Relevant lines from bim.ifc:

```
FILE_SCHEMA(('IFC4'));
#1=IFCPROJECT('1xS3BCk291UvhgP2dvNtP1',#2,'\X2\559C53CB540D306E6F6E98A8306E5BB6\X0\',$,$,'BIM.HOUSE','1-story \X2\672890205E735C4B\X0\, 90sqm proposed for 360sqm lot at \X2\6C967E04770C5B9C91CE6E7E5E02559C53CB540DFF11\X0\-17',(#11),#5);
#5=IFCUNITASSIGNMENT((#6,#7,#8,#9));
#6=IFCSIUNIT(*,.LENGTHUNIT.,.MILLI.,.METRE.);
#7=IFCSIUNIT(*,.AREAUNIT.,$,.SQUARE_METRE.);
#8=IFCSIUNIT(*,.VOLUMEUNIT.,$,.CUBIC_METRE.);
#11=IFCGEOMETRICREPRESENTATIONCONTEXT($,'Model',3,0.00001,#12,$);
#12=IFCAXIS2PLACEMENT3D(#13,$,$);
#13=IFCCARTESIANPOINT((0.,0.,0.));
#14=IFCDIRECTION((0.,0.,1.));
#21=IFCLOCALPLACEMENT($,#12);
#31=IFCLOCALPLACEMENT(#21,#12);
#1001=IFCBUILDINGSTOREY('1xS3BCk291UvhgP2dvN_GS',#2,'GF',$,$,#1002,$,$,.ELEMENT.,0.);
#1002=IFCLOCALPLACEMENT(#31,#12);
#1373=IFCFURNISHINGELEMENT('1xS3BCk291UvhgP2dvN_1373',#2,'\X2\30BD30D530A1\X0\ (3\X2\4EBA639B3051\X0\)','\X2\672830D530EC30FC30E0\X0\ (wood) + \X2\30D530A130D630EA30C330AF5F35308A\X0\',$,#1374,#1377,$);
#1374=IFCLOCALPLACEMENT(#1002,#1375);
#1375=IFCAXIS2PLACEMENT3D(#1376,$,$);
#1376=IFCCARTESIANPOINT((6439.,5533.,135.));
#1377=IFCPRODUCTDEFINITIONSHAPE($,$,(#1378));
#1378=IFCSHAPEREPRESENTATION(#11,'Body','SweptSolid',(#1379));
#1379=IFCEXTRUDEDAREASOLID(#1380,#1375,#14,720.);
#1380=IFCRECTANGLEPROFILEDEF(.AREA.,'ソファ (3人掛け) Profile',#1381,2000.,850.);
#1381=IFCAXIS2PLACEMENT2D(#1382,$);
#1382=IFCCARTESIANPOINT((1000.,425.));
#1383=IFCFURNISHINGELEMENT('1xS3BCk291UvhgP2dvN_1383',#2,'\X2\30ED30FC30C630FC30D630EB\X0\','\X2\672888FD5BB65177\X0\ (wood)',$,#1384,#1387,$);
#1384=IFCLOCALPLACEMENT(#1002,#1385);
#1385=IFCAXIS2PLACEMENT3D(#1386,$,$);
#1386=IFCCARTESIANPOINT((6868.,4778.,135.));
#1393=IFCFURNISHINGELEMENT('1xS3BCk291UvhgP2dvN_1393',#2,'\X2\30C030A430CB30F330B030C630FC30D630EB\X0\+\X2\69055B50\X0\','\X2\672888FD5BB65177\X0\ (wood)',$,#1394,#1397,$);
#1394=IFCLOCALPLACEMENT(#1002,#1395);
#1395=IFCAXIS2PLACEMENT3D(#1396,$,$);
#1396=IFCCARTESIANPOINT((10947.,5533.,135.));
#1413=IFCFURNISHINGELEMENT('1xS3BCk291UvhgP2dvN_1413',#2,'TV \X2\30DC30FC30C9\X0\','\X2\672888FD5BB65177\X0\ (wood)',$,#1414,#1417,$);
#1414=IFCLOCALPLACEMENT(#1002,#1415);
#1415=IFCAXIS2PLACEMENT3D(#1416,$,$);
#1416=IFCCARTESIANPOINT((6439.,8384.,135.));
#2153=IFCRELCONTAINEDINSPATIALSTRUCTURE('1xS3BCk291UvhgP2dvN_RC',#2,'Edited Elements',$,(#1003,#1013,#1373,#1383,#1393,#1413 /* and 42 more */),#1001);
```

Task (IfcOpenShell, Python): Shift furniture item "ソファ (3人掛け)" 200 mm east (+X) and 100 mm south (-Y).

```python
import ifcopenshell
import ifcopenshell.api.geometry
import ifcopenshell.util.placement
import ifcopenshell.util.unit

model = ifcopenshell.open("bim.ifc")
unit_scale = ifcopenshell.util.unit.calculate_unit_scale(model)

item = model.by_guid("1xS3BCk291UvhgP2dvN_1373")
matrix = ifcopenshell.util.placement.get_local_placement(item.ObjectPlacement)
matrix[0, 3] += 0.2 / unit_scale
matrix[1, 3] -= 0.1 / unit_scale
ifcopenshell.api.geometry.edit_object_placement(model, product=item, matrix=matrix, is_si=False)

print(ifcopenshell.util.placement.get_local_placement(item.ObjectPlacement).round(3) + 0.0)

model.write("bim_v2.ifc")
```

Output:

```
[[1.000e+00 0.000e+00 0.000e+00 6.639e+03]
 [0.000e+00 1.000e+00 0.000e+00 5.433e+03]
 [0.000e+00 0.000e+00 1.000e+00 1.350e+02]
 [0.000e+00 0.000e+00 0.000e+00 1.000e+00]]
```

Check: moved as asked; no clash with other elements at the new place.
